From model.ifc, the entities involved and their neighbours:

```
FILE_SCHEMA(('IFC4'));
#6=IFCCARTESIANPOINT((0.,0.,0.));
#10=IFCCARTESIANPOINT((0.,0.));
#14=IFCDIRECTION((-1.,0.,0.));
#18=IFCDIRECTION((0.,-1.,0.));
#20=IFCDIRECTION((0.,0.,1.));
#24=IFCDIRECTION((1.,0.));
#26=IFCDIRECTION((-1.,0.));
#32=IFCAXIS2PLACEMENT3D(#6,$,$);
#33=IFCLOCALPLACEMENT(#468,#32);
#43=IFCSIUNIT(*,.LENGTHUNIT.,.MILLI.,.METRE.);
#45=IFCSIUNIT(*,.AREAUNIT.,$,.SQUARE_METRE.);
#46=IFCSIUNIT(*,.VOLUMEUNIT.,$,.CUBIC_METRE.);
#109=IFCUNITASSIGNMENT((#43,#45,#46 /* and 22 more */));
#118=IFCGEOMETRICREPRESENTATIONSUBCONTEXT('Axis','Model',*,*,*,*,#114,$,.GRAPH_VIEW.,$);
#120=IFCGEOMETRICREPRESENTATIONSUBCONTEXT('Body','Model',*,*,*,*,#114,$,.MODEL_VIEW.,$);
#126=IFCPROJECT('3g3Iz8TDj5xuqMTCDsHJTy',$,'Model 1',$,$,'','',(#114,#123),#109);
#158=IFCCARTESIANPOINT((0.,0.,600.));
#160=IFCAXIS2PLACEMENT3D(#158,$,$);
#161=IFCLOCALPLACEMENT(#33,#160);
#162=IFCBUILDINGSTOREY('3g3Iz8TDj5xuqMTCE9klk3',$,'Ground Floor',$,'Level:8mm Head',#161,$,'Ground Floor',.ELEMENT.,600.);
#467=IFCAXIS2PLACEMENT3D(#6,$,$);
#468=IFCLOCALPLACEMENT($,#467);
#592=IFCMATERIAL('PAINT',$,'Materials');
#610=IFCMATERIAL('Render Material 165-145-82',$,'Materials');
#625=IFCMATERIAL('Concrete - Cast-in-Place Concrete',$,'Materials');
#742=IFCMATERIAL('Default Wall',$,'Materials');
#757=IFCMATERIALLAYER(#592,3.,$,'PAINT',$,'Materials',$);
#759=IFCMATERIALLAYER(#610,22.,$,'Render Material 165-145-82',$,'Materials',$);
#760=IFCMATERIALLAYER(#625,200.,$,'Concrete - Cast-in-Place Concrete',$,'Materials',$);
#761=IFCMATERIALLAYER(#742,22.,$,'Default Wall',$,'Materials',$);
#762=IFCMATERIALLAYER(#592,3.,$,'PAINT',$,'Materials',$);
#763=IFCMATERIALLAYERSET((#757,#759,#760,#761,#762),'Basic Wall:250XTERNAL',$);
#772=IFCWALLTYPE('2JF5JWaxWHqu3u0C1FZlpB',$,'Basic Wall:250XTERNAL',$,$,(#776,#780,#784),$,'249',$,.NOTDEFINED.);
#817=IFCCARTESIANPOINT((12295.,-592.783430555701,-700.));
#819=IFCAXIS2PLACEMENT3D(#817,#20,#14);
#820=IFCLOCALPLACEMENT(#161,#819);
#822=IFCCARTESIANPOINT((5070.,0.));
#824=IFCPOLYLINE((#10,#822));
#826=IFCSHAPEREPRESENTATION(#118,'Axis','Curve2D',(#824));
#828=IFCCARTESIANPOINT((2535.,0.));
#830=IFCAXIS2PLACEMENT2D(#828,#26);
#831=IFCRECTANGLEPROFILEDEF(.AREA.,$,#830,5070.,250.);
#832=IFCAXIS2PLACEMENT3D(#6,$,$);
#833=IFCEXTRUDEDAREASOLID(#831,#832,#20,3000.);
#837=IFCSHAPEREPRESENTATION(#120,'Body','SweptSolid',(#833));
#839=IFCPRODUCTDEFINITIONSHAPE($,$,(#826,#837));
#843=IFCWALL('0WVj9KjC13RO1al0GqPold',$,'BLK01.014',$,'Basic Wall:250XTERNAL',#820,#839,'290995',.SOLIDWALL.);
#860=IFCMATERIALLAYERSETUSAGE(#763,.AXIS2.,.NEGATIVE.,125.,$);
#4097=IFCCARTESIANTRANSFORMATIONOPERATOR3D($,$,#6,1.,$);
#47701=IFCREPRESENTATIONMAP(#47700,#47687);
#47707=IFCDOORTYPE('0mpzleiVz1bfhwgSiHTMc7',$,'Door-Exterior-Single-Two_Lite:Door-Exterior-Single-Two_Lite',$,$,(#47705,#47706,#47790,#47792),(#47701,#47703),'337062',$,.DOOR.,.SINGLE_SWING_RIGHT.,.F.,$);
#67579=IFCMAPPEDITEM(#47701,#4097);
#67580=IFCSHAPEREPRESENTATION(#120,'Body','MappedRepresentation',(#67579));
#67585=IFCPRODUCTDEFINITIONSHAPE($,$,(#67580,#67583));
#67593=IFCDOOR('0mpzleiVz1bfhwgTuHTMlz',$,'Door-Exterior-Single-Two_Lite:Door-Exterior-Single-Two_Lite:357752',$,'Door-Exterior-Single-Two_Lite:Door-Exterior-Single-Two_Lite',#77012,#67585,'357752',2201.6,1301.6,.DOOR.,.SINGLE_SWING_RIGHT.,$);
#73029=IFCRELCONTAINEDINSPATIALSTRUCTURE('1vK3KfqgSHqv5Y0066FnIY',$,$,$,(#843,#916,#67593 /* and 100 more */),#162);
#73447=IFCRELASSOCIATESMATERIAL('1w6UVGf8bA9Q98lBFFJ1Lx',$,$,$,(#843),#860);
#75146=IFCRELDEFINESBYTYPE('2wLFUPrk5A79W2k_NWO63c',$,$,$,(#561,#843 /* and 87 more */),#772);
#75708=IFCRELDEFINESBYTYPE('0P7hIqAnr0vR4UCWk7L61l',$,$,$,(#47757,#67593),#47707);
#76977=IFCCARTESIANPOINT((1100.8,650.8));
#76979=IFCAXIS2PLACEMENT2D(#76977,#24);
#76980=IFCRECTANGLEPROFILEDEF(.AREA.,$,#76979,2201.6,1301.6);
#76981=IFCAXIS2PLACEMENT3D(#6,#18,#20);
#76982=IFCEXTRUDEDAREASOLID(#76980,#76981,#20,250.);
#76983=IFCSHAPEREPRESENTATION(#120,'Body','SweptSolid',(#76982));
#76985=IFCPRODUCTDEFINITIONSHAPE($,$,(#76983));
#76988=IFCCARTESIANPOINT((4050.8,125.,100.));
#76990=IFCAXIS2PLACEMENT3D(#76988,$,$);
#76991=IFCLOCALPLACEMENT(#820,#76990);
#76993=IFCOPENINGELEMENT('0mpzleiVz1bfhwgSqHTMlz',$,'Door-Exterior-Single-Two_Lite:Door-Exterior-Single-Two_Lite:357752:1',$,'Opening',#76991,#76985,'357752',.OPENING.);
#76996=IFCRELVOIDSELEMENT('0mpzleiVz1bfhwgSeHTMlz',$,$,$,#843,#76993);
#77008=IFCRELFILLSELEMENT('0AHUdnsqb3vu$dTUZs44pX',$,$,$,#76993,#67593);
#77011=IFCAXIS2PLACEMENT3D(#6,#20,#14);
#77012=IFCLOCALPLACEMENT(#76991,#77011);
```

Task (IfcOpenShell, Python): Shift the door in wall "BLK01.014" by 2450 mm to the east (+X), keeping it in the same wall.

```python
import ifcopenshell
import ifcopenshell.api.geometry
import ifcopenshell.util.placement
import ifcopenshell.util.unit

model = ifcopenshell.open("model.ifc")
unit_scale = ifcopenshell.util.unit.calculate_unit_scale(model)

door = model.by_guid("0mpzleiVz1bfhwgTuHTMlz")
opening = door.FillsVoids[0].RelatingOpeningElement
wall = opening.VoidsElements[0].RelatingBuildingElement

wall_matrix = ifcopenshell.util.placement.get_local_placement(wall.ObjectPlacement)
shift = wall_matrix[:3, 0] * -2.45 / unit_scale
before = ifcopenshell.util.placement.get_local_placement(door.ObjectPlacement)[:3, 3].copy()

# The door is placed relative to its opening, so it follows when the opening moves.
matrix = ifcopenshell.util.placement.get_local_placement(opening.ObjectPlacement)
matrix[:3, 3] += shift
ifcopenshell.api.geometry.edit_object_placement(
    model, product=opening, matrix=matrix, is_si=False, should_transform_children=True
)

after = ifcopenshell.util.placement.get_local_placement(door.ObjectPlacement)[:3, 3]
print("door moved by", (after - before).round(3) + 0.0)

model.write("model_v2.ifc")
```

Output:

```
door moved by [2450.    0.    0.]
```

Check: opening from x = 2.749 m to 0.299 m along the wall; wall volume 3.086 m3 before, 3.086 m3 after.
